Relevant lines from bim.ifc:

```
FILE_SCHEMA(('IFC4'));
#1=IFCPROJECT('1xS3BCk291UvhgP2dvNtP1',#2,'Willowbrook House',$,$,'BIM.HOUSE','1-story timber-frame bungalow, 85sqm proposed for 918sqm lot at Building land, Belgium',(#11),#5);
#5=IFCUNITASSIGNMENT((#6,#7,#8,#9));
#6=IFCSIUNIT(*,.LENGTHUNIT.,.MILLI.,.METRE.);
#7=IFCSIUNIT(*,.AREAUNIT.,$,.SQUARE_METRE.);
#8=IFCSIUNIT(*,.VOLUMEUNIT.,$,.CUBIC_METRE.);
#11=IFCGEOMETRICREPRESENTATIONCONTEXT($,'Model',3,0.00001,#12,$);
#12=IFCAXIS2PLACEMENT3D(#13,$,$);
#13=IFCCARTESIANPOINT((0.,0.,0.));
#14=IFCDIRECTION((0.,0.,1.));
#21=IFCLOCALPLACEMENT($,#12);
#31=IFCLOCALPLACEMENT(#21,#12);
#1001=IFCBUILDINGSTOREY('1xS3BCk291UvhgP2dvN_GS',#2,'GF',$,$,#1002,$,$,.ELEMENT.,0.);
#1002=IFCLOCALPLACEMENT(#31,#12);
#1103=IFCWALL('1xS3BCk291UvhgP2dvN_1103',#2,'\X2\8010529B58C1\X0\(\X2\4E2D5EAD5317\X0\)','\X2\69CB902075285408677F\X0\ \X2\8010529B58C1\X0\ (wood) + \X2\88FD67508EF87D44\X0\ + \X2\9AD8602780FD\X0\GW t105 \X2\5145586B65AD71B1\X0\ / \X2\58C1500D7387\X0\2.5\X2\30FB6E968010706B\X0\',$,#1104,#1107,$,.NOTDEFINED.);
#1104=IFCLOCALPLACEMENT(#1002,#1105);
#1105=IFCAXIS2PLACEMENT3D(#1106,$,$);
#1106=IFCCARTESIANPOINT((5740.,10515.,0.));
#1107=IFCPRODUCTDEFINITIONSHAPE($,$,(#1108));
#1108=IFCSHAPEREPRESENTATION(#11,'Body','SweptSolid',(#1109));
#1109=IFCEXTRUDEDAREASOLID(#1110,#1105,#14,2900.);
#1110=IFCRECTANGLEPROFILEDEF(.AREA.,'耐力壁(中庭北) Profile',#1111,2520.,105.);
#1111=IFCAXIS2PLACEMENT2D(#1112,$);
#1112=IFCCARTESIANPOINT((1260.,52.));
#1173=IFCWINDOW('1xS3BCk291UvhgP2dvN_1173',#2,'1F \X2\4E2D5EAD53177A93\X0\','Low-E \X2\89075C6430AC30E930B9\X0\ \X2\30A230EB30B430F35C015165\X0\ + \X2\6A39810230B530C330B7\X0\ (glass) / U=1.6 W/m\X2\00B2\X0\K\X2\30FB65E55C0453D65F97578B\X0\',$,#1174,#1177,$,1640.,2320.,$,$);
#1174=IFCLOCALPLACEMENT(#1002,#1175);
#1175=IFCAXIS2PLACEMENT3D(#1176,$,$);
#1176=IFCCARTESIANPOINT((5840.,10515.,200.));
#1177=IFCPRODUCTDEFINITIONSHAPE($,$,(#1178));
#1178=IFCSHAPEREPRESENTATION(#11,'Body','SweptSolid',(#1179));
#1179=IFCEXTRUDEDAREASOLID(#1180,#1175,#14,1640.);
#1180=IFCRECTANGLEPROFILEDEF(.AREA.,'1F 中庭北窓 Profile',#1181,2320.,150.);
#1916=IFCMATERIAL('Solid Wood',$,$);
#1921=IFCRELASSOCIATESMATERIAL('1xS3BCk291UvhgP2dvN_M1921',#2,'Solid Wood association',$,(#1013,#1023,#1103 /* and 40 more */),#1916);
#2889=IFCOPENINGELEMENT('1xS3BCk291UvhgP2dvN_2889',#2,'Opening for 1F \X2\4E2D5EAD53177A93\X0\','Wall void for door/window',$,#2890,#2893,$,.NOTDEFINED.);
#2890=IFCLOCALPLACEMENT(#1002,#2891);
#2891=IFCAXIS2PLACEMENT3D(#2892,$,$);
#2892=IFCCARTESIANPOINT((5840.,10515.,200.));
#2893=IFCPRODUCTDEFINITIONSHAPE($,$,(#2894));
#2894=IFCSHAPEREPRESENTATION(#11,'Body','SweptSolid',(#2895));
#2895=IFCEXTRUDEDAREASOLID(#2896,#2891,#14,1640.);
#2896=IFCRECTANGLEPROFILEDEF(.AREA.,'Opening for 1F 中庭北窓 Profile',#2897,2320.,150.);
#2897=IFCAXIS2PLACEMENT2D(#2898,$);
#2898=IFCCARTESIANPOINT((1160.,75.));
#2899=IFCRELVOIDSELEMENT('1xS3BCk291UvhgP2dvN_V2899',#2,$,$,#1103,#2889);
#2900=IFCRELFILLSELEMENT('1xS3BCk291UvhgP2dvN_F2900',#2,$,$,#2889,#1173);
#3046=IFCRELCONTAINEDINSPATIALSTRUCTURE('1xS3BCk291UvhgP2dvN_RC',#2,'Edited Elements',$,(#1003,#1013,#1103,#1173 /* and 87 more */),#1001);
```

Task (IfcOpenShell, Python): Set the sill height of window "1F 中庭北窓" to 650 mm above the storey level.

```python
import numpy as np
import ifcopenshell
import ifcopenshell.api.geometry
import ifcopenshell.geom
import ifcopenshell.util.element
import ifcopenshell.util.placement
import ifcopenshell.util.shape
import ifcopenshell.util.unit

model = ifcopenshell.open("bim.ifc")
unit_scale = ifcopenshell.util.unit.calculate_unit_scale(model)

window = model.by_id(1173)
opening = window.FillsVoids[0].RelatingOpeningElement
storey = ifcopenshell.util.element.get_container(window, ifc_class="IfcBuildingStorey")
level = ifcopenshell.util.placement.get_local_placement(storey.ObjectPlacement)[2, 3]

# The opening's origin need not be at the sill, so measure its lowest point.
shape = ifcopenshell.geom.create_shape(ifcopenshell.geom.settings(), opening)
bottom = ifcopenshell.util.shape.get_shape_bottom_elevation(shape, shape.geometry) / unit_scale
dz = level + 650.0 - bottom

shift = np.array([0.0, 0.0, dz])
# The window is not placed relative to its opening, so move both.
for product in (opening, window):
    matrix = ifcopenshell.util.placement.get_local_placement(product.ObjectPlacement)
    matrix[:3, 3] += shift
    ifcopenshell.api.geometry.edit_object_placement(model, product=product, matrix=matrix, is_si=False)

print(f"moved by {dz * unit_scale:+.3f} m")

model.write("bim-out.ifc")
```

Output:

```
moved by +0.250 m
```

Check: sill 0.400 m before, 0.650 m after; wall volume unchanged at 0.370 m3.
